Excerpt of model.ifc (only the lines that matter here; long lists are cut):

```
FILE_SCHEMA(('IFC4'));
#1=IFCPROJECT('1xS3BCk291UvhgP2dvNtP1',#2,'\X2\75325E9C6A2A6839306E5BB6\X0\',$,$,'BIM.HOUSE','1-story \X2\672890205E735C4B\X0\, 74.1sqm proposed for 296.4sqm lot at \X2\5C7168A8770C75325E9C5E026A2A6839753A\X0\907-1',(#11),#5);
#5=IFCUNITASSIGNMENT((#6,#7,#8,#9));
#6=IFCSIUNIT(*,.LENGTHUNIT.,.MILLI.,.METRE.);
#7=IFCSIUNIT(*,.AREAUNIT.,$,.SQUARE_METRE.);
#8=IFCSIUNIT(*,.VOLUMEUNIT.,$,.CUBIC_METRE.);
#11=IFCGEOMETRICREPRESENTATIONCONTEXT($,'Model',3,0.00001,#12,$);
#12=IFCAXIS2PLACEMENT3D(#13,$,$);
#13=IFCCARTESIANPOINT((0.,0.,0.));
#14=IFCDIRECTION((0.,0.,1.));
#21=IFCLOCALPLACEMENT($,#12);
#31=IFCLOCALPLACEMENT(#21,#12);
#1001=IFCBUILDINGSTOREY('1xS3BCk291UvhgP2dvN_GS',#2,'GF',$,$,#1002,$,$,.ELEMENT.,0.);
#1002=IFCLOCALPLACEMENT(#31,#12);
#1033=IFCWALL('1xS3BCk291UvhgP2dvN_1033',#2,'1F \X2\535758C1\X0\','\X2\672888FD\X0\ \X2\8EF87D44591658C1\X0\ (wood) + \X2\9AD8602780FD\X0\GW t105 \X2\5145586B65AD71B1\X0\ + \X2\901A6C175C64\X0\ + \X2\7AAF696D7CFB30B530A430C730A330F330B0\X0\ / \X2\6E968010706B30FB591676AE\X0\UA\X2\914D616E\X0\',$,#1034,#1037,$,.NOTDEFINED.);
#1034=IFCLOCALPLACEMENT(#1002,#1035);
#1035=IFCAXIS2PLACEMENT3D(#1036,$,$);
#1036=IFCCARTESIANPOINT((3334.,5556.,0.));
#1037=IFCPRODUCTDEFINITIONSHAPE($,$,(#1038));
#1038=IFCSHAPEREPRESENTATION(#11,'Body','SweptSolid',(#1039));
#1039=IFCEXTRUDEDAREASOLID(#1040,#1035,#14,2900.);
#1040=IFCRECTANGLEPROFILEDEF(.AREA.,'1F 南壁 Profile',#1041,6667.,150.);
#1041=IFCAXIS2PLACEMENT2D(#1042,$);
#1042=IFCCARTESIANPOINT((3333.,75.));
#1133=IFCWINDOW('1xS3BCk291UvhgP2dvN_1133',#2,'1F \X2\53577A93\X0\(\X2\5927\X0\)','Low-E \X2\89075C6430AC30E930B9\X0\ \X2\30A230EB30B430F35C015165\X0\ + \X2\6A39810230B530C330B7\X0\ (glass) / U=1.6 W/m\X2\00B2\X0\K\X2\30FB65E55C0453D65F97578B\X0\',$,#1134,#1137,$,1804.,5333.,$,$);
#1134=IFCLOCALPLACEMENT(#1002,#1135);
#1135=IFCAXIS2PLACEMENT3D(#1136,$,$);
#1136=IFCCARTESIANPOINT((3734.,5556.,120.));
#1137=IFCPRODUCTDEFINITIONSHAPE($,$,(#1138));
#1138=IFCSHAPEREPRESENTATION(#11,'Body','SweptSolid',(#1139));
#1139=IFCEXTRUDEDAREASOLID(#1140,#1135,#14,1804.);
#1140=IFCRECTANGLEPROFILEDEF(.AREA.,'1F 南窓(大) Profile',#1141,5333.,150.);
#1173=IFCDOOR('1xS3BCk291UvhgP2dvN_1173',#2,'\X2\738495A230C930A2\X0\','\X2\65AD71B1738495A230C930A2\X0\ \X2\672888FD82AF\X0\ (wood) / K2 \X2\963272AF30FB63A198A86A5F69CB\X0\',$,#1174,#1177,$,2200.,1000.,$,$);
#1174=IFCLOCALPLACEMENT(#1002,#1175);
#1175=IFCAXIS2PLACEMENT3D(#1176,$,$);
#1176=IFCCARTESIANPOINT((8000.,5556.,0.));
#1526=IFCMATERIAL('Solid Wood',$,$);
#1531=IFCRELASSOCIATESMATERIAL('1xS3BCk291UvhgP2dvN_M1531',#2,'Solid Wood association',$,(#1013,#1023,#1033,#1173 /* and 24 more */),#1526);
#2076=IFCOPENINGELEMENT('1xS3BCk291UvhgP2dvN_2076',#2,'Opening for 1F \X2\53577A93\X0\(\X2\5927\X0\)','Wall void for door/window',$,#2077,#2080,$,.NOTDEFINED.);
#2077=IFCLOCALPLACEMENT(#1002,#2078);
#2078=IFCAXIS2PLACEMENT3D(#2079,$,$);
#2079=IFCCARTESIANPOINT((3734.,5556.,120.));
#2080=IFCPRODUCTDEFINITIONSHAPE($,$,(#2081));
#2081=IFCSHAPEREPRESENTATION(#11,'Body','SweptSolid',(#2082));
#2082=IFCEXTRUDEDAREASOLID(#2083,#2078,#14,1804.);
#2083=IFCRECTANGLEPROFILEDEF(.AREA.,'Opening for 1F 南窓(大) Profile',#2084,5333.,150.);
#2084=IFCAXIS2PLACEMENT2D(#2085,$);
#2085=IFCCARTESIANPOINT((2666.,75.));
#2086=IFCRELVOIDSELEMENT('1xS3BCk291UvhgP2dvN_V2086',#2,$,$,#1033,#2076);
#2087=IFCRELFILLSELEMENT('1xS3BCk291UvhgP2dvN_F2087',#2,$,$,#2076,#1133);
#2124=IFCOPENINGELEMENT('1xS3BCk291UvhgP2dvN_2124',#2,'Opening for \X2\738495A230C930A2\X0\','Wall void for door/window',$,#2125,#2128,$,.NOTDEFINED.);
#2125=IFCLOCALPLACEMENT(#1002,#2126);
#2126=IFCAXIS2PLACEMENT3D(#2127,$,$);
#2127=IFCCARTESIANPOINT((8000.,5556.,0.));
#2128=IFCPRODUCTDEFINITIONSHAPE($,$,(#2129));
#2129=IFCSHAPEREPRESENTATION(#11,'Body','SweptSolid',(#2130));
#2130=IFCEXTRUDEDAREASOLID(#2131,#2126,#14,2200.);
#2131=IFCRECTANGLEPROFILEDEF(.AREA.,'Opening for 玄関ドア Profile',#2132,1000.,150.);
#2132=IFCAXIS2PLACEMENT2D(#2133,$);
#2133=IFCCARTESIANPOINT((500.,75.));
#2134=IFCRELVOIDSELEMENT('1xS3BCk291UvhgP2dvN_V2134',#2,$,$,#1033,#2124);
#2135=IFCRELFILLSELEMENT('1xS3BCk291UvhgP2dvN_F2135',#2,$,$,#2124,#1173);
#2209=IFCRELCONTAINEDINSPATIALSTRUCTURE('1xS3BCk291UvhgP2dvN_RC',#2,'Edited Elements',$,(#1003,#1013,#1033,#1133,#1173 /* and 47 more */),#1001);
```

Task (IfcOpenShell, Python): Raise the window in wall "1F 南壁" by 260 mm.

```python
import numpy as np
import ifcopenshell
import ifcopenshell.api.geometry
import ifcopenshell.util.placement
import ifcopenshell.util.unit

model = ifcopenshell.open("model.ifc")
unit_scale = ifcopenshell.util.unit.calculate_unit_scale(model)

window = model.by_guid("1xS3BCk291UvhgP2dvN_1133")
opening = window.FillsVoids[0].RelatingOpeningElement
dz = 0.26 / unit_scale

shift = np.array([0.0, 0.0, dz])
# The window is not placed relative to its opening, so move both.
for product in (opening, window):
    matrix = ifcopenshell.util.placement.get_local_placement(product.ObjectPlacement)
    matrix[:3, 3] += shift
    ifcopenshell.api.geometry.edit_object_placement(model, product=product, matrix=matrix, is_si=False)

print(f"moved by {dz * unit_scale:+.3f} m")

model.write("model_v2.ifc")
```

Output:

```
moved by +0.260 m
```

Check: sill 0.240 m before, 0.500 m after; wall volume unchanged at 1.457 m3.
